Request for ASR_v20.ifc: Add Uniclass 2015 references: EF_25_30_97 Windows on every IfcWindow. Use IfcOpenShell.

First a look at what the model holds.

```python
import ifcopenshell

model = ifcopenshell.open("ASR_v20.ifc")
print(model.schema)
print("classifications:", [c.Name for c in model.by_type("IfcClassification")])
for ifc_class in ("IfcDoor", "IfcRoof", "IfcStair", "IfcWall", "IfcWindow"):
    print(ifc_class, len(model.by_type(ifc_class)))
```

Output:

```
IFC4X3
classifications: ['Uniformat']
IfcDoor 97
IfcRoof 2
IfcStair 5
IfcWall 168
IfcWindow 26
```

```python
import ifcopenshell
import ifcopenshell.api.classification

model = ifcopenshell.open("ASR_v20.ifc")

system = ifcopenshell.api.classification.add_classification(model, classification="Uniclass 2015")

codes = {
    "IfcWindow": ("EF_25_30_97", "Windows"),
}
for ifc_class, (code, name) in codes.items():
    products = model.by_type(ifc_class)
    ifcopenshell.api.classification.add_reference(
        model, products=products, classification=system, identification=code, name=name
    )
    print(code, len(products))

model.write("ASR_v20_updated.ifc")
```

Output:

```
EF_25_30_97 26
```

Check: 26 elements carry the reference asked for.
